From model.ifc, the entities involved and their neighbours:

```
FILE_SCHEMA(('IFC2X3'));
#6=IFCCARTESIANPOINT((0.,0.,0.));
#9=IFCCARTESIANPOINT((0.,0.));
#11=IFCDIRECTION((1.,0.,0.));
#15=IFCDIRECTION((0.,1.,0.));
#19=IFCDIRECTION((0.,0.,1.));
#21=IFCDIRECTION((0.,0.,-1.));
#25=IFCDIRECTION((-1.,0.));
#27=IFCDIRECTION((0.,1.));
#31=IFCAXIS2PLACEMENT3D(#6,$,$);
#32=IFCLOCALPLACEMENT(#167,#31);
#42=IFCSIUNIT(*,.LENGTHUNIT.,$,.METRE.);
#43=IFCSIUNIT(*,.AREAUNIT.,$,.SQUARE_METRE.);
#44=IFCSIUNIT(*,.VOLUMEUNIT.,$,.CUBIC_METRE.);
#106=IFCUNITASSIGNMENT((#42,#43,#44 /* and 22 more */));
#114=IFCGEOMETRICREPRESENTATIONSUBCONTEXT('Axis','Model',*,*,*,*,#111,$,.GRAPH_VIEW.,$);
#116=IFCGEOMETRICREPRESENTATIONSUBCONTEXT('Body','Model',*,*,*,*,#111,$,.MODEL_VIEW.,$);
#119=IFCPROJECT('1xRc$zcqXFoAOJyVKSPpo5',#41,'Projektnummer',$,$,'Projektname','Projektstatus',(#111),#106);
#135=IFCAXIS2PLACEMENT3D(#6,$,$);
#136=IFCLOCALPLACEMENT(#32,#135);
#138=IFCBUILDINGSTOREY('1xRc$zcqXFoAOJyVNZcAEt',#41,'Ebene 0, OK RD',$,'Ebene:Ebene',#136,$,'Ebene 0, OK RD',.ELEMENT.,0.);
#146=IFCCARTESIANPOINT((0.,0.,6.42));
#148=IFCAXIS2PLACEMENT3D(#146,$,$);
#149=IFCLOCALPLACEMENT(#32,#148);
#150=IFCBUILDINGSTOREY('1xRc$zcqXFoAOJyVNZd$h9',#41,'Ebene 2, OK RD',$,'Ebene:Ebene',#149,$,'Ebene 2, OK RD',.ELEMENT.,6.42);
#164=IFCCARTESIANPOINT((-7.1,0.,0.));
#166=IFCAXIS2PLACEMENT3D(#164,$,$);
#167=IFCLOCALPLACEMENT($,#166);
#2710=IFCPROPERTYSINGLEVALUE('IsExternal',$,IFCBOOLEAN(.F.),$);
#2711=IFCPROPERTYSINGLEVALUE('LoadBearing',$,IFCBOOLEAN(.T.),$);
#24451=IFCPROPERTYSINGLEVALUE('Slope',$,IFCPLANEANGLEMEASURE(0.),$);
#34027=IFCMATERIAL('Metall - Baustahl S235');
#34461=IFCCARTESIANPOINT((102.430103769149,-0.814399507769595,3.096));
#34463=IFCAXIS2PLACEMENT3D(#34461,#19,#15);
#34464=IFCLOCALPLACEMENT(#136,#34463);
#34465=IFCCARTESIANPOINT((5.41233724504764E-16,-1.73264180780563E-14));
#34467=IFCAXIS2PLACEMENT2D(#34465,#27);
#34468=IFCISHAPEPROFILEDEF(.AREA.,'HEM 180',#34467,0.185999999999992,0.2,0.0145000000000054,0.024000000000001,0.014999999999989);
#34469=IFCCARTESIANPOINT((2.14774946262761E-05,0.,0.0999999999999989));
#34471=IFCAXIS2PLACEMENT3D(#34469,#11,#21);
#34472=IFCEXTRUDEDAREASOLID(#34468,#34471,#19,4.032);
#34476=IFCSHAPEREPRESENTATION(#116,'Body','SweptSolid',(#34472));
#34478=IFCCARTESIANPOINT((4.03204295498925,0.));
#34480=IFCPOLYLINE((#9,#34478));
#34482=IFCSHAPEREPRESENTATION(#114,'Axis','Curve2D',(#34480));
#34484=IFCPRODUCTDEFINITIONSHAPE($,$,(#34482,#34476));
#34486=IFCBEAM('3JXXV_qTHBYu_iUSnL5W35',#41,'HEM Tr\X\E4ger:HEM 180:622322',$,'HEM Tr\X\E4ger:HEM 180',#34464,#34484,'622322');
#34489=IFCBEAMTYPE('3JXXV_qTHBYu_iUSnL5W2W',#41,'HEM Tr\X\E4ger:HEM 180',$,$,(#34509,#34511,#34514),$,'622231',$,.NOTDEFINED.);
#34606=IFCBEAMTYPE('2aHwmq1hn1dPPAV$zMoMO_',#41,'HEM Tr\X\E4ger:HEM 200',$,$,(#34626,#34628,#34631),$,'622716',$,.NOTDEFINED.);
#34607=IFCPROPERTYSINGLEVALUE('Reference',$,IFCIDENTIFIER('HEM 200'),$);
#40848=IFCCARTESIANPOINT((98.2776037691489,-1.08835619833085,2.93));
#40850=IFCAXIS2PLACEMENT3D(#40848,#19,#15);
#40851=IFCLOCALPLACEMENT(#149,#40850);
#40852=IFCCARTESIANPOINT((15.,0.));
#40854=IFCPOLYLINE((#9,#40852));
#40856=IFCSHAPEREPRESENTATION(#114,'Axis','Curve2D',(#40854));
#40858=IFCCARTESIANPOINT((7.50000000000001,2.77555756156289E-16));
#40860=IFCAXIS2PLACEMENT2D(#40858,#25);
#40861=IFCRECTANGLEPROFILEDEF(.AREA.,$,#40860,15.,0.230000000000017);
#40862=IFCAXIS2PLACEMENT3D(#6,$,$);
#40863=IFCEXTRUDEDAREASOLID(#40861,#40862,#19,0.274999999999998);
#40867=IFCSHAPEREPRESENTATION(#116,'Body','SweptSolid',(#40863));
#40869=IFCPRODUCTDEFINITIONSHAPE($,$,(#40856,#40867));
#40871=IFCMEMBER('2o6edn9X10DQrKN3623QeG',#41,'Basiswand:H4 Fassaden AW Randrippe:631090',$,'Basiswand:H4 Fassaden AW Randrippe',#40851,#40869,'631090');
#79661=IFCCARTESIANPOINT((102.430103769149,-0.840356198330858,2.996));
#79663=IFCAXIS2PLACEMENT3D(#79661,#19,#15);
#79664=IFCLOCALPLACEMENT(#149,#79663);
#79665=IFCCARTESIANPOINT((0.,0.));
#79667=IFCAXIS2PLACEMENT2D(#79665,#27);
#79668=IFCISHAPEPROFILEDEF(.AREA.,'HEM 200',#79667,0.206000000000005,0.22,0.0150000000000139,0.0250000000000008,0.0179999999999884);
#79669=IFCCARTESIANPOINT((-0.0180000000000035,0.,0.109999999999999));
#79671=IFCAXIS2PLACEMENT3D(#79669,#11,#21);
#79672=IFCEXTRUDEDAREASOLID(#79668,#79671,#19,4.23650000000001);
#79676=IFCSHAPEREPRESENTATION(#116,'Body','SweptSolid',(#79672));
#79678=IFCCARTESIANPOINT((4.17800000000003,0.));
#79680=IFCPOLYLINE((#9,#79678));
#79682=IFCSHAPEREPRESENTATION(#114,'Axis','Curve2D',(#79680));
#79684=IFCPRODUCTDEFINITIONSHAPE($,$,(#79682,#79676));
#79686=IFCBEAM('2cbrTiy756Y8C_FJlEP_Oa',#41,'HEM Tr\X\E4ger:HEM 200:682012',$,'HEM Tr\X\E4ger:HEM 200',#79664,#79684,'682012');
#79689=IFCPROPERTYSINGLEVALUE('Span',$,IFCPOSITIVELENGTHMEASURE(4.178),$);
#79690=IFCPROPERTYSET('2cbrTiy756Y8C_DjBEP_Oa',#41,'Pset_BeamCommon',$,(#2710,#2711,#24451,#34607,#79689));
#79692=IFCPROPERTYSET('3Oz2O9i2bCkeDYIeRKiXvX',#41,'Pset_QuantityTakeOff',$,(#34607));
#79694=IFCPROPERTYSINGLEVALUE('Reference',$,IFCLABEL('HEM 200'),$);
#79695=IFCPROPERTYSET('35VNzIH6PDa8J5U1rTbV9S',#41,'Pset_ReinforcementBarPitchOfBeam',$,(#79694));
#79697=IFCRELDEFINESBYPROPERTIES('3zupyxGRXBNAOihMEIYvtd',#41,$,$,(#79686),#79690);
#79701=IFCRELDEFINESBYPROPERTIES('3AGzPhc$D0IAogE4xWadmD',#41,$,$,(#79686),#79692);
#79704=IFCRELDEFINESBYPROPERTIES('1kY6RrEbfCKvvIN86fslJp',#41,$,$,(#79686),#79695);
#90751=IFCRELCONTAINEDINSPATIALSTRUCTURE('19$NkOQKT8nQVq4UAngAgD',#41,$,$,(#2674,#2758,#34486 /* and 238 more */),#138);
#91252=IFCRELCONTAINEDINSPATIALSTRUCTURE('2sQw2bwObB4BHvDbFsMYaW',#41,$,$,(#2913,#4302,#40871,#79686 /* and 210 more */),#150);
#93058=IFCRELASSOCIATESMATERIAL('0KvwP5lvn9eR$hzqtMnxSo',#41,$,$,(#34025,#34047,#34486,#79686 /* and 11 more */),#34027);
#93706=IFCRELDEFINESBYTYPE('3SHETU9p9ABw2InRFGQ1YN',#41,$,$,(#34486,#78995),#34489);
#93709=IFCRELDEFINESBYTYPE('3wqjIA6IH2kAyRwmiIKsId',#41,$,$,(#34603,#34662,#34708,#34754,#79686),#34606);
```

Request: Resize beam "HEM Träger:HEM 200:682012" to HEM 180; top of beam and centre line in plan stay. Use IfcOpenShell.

```python
import ifcopenshell
import ifcopenshell.api.pset
import ifcopenshell.api.type
import ifcopenshell.util.element
import ifcopenshell.util.representation

model = ifcopenshell.open("model.ifc")

member = model.by_guid("2cbrTiy756Y8C_FJlEP_Oa")
source = next(p for p in model.by_type("IfcIShapeProfileDef") if p.ProfileName == "HEM 180")

body = ifcopenshell.util.representation.get_representation(member, "Model", "Body")
solid = body.Items[0]
old_profile = solid.SweptArea

# Copy the section's sizes but keep this member's own profile position.
profile = ifcopenshell.util.element.copy(model, source)
# Profiles are centred, so shift by half the change in depth to hold the top.
shift = (old_profile.OverallDepth - profile.OverallDepth) / 2
x, y = old_profile.Position.Location.Coordinates
up = (-1.0, 0.0)  # upwards, in the solid's own plane
location = model.createIfcCartesianPoint((x + up[0] * shift, y + up[1] * shift))
profile.Position = model.createIfcAxis2Placement2D(location, old_profile.Position.RefDirection)
solid.SweptArea = profile
if not model.get_total_inverses(old_profile):
    ifcopenshell.util.element.remove_deep2(model, old_profile)

new_type = model.by_guid("3JXXV_qTHBYu_iUSnL5W2W")
ifcopenshell.api.type.assign_type(
    model, related_objects=[member], relating_type=new_type, should_map_representations=False
)
member.Name = member.Name.replace("HEM 200", "HEM 180")
member.ObjectType = "HEM Träger:HEM 180"
pset = model.by_id(ifcopenshell.util.element.get_pset(member, "Pset_BeamCommon", should_inherit=False)["id"])
ifcopenshell.api.pset.edit_pset(model, pset=pset, properties={"Reference": "HEM 180"})
pset = model.by_id(ifcopenshell.util.element.get_pset(member, "Pset_QuantityTakeOff", should_inherit=False)["id"])
ifcopenshell.api.pset.edit_pset(model, pset=pset, properties={"Reference": "HEM 180"})
pset = model.by_id(ifcopenshell.util.element.get_pset(member, "Pset_ReinforcementBarPitchOfBeam", should_inherit=False)["id"])
ifcopenshell.api.pset.edit_pset(model, pset=pset, properties={"Reference": "HEM 180"})

print(solid.SweptArea)

model.write("model_v2.ifc")
```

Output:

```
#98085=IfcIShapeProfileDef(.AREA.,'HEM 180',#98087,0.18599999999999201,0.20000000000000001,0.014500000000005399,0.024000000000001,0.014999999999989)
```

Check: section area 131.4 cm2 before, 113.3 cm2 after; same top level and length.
